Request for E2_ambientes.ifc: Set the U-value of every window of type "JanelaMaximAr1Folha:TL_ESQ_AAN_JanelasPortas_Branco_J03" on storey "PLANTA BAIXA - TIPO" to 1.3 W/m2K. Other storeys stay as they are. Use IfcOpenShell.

First a look at what the model holds.

```python
import ifcopenshell
import ifcopenshell.util.element

model = ifcopenshell.open("E2_ambientes.ifc")
print(model.schema)
storey = next(s for s in model.by_type("IfcBuildingStorey") if s.Name == "PLANTA BAIXA - TIPO")
windows = [e for e in ifcopenshell.util.element.get_decomposition(storey) if e.is_a("IfcWindow")]
seen = {}
for e in windows:
    element_type = ifcopenshell.util.element.get_type(e)
    key = (element_type.Name if element_type != e and element_type else None, ifcopenshell.util.element.get_pset(e, "Pset_WindowCommon", "ThermalTransmittance"))
    seen[key] = seen.get(key, 0) + 1
for (name, value), count in sorted(seen.items(), key=str):
    print(count, "x", name, "|", value)
```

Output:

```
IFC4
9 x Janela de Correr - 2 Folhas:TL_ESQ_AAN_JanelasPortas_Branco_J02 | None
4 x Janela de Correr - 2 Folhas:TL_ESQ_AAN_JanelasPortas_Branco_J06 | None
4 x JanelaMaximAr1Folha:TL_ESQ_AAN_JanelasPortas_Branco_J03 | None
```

```python
import ifcopenshell
import ifcopenshell.api.pset
import ifcopenshell.util.element

model = ifcopenshell.open("E2_ambientes.ifc")

storey = next(s for s in model.by_type("IfcBuildingStorey") if s.Name == "PLANTA BAIXA - TIPO")
windows = [e for e in ifcopenshell.util.element.get_decomposition(storey) if e.is_a("IfcWindow")]

count = 0
for e in windows:
    element_type = ifcopenshell.util.element.get_type(e)
    if element_type in (None, e) or element_type.Name != "JanelaMaximAr1Folha:TL_ESQ_AAN_JanelasPortas_Branco_J03":
        continue
    # add_pset returns the element's existing set when there is one.
    pset = ifcopenshell.api.pset.add_pset(model, product=e, name="Pset_WindowCommon")
    ifcopenshell.api.pset.edit_pset(model, pset=pset, properties={"ThermalTransmittance": 1.3})
    count += 1

print(count, "windows updated")

model.write("E2_ambientes-out.ifc")
```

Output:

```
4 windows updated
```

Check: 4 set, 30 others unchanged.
